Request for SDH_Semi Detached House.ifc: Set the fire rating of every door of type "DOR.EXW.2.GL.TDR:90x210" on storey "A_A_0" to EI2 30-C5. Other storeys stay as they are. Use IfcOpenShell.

First a look at what the model holds.

```python
import ifcopenshell
import ifcopenshell.util.element

model = ifcopenshell.open("SDH_Semi Detached House.ifc")
print(model.schema)
storey = next(s for s in model.by_type("IfcBuildingStorey") if s.Name == "A_A_0")
doors = [e for e in ifcopenshell.util.element.get_decomposition(storey) if e.is_a("IfcDoor")]
seen = {}
for e in doors:
    element_type = ifcopenshell.util.element.get_type(e)
    key = (element_type.Name if element_type != e and element_type else None, ifcopenshell.util.element.get_pset(e, "Pset_DoorCommon", "FireRating"))
    seen[key] = seen.get(key, 0) + 1
for (name, value), count in sorted(seen.items(), key=str):
    print(count, "x", name, "|", value)
```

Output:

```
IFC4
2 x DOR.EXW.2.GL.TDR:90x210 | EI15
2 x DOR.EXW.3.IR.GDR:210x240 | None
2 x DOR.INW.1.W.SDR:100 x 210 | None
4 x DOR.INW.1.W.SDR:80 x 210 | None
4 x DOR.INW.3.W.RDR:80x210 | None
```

```python
import ifcopenshell
import ifcopenshell.api.pset
import ifcopenshell.util.element

model = ifcopenshell.open("SDH_Semi Detached House.ifc")

storey = next(s for s in model.by_type("IfcBuildingStorey") if s.Name == "A_A_0")
doors = [e for e in ifcopenshell.util.element.get_decomposition(storey) if e.is_a("IfcDoor")]

count = 0
for e in doors:
    element_type = ifcopenshell.util.element.get_type(e)
    if element_type in (None, e) or element_type.Name != "DOR.EXW.2.GL.TDR:90x210":
        continue
    # add_pset returns the element's existing set when there is one.
    pset = ifcopenshell.api.pset.add_pset(model, product=e, name="Pset_DoorCommon")
    ifcopenshell.api.pset.edit_pset(model, pset=pset, properties={"FireRating": "EI2 30-C5"})
    count += 1

print(count, "doors updated")

model.write("SDH_Semi Detached House_v2.ifc")
```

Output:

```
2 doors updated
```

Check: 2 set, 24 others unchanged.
